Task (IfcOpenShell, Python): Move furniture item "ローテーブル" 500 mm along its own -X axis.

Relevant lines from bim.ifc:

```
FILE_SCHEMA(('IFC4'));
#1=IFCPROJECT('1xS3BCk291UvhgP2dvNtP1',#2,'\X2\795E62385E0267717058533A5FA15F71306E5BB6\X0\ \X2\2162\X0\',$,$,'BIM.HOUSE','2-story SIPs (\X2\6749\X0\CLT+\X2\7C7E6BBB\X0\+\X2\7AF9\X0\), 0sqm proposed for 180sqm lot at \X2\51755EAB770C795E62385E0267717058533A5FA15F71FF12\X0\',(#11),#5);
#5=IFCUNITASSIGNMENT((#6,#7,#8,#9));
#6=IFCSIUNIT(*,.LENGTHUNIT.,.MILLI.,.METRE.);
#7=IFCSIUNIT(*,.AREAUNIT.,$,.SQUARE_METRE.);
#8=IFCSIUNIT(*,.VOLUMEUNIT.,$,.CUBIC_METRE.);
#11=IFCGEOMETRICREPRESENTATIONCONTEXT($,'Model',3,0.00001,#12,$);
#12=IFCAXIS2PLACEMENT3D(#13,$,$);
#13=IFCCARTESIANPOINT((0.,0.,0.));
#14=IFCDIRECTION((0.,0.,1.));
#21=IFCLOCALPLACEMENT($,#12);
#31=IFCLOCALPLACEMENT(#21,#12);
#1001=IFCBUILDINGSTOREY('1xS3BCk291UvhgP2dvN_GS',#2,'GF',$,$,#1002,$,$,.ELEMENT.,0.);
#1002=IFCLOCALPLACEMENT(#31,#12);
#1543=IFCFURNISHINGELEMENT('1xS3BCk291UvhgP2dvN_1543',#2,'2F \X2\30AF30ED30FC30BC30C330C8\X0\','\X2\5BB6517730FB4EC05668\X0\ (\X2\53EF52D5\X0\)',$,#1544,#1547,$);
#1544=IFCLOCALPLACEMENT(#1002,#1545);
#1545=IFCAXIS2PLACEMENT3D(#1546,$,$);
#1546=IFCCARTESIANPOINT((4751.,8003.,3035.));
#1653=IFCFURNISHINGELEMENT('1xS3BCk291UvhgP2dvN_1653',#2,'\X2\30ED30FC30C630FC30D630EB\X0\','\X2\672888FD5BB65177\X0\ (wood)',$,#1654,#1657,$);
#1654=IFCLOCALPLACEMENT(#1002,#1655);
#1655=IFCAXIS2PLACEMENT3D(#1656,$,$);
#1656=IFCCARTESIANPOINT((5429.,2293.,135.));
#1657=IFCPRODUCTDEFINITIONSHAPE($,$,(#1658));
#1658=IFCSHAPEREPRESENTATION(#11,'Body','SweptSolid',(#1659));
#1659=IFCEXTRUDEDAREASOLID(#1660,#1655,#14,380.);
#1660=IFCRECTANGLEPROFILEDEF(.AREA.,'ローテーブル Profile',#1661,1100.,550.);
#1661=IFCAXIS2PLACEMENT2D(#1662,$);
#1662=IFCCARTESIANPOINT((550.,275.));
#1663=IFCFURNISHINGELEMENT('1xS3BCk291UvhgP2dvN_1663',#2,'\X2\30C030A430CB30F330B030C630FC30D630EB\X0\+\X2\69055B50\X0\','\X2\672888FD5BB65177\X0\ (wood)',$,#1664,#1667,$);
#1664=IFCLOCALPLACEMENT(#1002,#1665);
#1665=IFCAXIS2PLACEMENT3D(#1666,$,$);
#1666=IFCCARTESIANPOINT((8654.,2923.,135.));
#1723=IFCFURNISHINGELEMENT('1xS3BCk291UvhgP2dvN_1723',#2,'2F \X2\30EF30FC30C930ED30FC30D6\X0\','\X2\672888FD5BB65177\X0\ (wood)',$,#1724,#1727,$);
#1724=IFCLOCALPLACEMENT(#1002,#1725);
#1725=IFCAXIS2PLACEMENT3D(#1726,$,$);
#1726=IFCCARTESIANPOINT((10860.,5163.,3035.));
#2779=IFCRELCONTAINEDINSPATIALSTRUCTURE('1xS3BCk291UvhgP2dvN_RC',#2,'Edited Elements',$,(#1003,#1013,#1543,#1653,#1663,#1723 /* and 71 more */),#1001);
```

```python
import ifcopenshell
import ifcopenshell.api.geometry
import ifcopenshell.util.placement

model = ifcopenshell.open("bim.ifc")

item = model.by_id(1653)
matrix = ifcopenshell.util.placement.get_local_placement(item.ObjectPlacement)
matrix[:3, 3] -= matrix[:3, 0] * 500.0
ifcopenshell.api.geometry.edit_object_placement(model, product=item, matrix=matrix, is_si=False)

print(ifcopenshell.util.placement.get_local_placement(item.ObjectPlacement).round(3) + 0.0)

model.write("bim_updated.ifc")
```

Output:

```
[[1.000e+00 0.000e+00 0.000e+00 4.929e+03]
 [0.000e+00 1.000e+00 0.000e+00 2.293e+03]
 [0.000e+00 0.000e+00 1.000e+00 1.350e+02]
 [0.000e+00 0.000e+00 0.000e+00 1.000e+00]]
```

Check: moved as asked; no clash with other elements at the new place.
